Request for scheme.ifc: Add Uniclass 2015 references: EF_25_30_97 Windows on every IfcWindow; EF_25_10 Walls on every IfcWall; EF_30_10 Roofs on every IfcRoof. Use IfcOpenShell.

First a look at what the model holds.

```python
import ifcopenshell

model = ifcopenshell.open("scheme.ifc")
print(model.schema)
print("classifications:", [c.Name for c in model.by_type("IfcClassification")])
for ifc_class in ("IfcDoor", "IfcRoof", "IfcStair", "IfcWall", "IfcWindow"):
    print(ifc_class, len(model.by_type(ifc_class)))
```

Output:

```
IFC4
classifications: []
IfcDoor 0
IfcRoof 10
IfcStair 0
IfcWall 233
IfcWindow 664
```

```python
import ifcopenshell
import ifcopenshell.api.classification

model = ifcopenshell.open("scheme.ifc")

system = ifcopenshell.api.classification.add_classification(model, classification="Uniclass 2015")

codes = {
    "IfcWindow": ("EF_25_30_97", "Windows"),
    "IfcWall": ("EF_25_10", "Walls"),
    "IfcRoof": ("EF_30_10", "Roofs"),
}
for ifc_class, (code, name) in codes.items():
    products = model.by_type(ifc_class)
    ifcopenshell.api.classification.add_reference(
        model, products=products, classification=system, identification=code, name=name
    )
    print(code, len(products))

model.write("scheme_rev.ifc")
```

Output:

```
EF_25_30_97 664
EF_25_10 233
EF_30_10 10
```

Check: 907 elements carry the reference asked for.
